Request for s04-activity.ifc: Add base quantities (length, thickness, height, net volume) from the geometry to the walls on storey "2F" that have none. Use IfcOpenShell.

First a look at what the model holds.

```python
import ifcopenshell
import ifcopenshell.util.element
import ifcopenshell.util.unit

model = ifcopenshell.open("s04-activity.ifc")
print(model.schema)
for unit_type in ("LENGTHUNIT", "AREAUNIT", "VOLUMEUNIT"):
    print(unit_type, ifcopenshell.util.unit.calculate_unit_scale(model, unit_type))
storey = next(s for s in model.by_type("IfcBuildingStorey") if s.Name == "2F")
walls = [e for e in ifcopenshell.util.element.get_decomposition(storey) if e.is_a("IfcWall")]
for e in sorted(walls, key=lambda e: e.id()):
    print(e.id(), e.is_a(), e.Name, list(ifcopenshell.util.element.get_psets(e, qtos_only=True)), sep=" | ")
```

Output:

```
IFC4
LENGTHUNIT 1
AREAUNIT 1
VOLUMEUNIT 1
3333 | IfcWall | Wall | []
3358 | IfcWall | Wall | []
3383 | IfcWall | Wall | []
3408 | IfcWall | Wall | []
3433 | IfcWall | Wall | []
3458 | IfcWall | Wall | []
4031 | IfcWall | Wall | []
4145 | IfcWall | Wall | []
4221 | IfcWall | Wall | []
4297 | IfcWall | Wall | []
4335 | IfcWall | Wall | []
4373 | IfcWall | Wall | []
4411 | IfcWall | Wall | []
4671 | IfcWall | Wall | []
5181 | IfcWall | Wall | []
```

```python
import ifcopenshell
import ifcopenshell.api.pset
import ifcopenshell.geom
import ifcopenshell.util.element
import ifcopenshell.util.shape
import ifcopenshell.util.unit

model = ifcopenshell.open("s04-activity.ifc")
unit_scale = ifcopenshell.util.unit.calculate_unit_scale(model)
volume_scale = ifcopenshell.util.unit.calculate_unit_scale(model, "VOLUMEUNIT")
settings = ifcopenshell.geom.settings()

storey = next(s for s in model.by_type("IfcBuildingStorey") if s.Name == "2F")
walls = [e for e in ifcopenshell.util.element.get_decomposition(storey) if e.is_a("IfcWall")]

for e in sorted(walls, key=lambda e: e.id()):
    if ifcopenshell.util.element.get_psets(e, qtos_only=True, should_inherit=False):
        continue
    # Geometry comes back in metres, in the element's own axes.
    shape = ifcopenshell.geom.create_shape(settings, e)
    values = {
        "Length": ifcopenshell.util.shape.get_x(shape.geometry) / unit_scale,
        "Width": ifcopenshell.util.shape.get_y(shape.geometry) / unit_scale,
        "Height": ifcopenshell.util.shape.get_z(shape.geometry) / unit_scale,
        "NetVolume": ifcopenshell.util.shape.get_volume(shape.geometry) / volume_scale,
    }
    qto = ifcopenshell.api.pset.add_qto(model, product=e, name="Qto_WallBaseQuantities")
    ifcopenshell.api.pset.edit_qto(model, qto=qto, properties=values)
    print(e.id(), {k: round(v, 3) for k, v in values.items()})

model.write("s04-activity_v2.ifc")
```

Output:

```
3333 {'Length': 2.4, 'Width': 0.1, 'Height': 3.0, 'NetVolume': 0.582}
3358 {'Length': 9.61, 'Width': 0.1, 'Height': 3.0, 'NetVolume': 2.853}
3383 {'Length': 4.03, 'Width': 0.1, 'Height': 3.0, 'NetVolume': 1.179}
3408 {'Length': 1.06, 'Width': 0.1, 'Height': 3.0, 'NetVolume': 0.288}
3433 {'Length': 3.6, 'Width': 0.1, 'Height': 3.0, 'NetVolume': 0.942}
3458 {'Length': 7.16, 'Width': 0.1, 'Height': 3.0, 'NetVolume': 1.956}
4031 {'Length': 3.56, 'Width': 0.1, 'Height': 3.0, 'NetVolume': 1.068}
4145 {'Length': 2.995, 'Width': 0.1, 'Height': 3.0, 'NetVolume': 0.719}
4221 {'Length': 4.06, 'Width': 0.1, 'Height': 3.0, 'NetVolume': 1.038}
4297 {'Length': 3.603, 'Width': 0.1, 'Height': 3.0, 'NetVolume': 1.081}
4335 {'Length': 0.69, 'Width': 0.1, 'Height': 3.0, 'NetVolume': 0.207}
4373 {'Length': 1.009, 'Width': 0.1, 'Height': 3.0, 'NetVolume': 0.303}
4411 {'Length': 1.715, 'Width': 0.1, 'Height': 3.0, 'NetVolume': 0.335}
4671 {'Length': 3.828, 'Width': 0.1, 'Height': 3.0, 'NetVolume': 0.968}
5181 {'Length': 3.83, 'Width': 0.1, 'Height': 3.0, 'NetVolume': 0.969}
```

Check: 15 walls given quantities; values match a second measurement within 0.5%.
